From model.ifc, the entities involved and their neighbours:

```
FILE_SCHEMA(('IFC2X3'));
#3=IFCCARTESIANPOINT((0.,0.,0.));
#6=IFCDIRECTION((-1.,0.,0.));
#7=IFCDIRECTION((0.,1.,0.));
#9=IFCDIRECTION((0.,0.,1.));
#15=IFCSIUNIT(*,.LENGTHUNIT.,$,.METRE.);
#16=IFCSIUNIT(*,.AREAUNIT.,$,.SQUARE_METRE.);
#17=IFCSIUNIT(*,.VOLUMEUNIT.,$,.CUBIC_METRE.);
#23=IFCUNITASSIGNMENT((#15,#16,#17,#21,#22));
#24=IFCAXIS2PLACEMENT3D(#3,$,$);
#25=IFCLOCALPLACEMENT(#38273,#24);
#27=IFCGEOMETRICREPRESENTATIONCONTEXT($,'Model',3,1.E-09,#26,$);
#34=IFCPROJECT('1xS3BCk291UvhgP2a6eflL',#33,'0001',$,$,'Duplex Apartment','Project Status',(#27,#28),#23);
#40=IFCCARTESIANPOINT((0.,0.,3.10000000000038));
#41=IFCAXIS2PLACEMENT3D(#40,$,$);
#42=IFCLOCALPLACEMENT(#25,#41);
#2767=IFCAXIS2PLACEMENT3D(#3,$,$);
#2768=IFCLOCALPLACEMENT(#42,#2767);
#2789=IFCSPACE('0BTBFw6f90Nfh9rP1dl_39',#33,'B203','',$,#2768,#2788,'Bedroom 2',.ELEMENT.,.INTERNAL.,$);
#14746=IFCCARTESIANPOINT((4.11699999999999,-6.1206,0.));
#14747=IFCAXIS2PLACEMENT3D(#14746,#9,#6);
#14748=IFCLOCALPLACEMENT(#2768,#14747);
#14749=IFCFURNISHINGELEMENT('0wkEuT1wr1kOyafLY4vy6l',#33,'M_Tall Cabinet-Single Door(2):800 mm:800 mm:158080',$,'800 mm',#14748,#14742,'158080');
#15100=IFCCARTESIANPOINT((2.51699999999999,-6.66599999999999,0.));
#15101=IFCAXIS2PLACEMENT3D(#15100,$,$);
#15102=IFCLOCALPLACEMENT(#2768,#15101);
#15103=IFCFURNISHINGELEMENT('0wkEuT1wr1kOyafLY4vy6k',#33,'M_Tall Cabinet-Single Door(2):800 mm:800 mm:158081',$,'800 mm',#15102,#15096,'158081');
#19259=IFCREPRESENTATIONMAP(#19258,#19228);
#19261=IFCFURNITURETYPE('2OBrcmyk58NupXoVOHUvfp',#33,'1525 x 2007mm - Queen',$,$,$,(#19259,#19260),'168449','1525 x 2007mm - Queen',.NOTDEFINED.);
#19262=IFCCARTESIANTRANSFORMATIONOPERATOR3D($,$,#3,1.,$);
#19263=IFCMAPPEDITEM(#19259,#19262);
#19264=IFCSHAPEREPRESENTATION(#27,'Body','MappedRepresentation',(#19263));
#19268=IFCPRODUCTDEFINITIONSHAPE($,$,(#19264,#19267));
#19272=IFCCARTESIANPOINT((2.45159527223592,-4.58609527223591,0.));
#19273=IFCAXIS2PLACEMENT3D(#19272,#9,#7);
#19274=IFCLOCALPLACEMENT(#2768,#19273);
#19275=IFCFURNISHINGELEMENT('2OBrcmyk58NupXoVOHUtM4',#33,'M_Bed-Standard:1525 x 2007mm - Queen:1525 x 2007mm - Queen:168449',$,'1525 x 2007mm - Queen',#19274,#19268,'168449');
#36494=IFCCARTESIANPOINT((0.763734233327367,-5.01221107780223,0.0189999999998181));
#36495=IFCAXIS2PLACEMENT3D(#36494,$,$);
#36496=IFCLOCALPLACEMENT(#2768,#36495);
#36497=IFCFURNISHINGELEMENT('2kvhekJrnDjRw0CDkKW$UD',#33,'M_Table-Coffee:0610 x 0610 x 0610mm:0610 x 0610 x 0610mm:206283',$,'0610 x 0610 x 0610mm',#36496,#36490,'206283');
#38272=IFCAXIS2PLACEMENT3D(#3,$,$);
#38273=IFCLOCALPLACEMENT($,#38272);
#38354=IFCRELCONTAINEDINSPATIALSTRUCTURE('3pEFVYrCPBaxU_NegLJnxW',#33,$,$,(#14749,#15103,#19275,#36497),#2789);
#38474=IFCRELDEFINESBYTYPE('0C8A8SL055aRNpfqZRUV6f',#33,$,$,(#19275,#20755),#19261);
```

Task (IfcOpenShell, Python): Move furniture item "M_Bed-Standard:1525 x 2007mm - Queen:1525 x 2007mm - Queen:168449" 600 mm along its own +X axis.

```python
import ifcopenshell
import ifcopenshell.api.geometry
import ifcopenshell.util.placement
import ifcopenshell.util.unit

model = ifcopenshell.open("model.ifc")
unit_scale = ifcopenshell.util.unit.calculate_unit_scale(model)

item = model.by_guid("2OBrcmyk58NupXoVOHUtM4")
matrix = ifcopenshell.util.placement.get_local_placement(item.ObjectPlacement)
matrix[:3, 3] += matrix[:3, 0] * 0.6 / unit_scale
ifcopenshell.api.geometry.edit_object_placement(model, product=item, matrix=matrix, is_si=False)

print(ifcopenshell.util.placement.get_local_placement(item.ObjectPlacement).round(3) + 0.0)

model.write("model-out.ifc")
```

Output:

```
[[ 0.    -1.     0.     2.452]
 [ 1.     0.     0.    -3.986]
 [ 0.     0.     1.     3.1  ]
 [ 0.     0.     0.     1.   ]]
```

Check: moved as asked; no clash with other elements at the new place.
